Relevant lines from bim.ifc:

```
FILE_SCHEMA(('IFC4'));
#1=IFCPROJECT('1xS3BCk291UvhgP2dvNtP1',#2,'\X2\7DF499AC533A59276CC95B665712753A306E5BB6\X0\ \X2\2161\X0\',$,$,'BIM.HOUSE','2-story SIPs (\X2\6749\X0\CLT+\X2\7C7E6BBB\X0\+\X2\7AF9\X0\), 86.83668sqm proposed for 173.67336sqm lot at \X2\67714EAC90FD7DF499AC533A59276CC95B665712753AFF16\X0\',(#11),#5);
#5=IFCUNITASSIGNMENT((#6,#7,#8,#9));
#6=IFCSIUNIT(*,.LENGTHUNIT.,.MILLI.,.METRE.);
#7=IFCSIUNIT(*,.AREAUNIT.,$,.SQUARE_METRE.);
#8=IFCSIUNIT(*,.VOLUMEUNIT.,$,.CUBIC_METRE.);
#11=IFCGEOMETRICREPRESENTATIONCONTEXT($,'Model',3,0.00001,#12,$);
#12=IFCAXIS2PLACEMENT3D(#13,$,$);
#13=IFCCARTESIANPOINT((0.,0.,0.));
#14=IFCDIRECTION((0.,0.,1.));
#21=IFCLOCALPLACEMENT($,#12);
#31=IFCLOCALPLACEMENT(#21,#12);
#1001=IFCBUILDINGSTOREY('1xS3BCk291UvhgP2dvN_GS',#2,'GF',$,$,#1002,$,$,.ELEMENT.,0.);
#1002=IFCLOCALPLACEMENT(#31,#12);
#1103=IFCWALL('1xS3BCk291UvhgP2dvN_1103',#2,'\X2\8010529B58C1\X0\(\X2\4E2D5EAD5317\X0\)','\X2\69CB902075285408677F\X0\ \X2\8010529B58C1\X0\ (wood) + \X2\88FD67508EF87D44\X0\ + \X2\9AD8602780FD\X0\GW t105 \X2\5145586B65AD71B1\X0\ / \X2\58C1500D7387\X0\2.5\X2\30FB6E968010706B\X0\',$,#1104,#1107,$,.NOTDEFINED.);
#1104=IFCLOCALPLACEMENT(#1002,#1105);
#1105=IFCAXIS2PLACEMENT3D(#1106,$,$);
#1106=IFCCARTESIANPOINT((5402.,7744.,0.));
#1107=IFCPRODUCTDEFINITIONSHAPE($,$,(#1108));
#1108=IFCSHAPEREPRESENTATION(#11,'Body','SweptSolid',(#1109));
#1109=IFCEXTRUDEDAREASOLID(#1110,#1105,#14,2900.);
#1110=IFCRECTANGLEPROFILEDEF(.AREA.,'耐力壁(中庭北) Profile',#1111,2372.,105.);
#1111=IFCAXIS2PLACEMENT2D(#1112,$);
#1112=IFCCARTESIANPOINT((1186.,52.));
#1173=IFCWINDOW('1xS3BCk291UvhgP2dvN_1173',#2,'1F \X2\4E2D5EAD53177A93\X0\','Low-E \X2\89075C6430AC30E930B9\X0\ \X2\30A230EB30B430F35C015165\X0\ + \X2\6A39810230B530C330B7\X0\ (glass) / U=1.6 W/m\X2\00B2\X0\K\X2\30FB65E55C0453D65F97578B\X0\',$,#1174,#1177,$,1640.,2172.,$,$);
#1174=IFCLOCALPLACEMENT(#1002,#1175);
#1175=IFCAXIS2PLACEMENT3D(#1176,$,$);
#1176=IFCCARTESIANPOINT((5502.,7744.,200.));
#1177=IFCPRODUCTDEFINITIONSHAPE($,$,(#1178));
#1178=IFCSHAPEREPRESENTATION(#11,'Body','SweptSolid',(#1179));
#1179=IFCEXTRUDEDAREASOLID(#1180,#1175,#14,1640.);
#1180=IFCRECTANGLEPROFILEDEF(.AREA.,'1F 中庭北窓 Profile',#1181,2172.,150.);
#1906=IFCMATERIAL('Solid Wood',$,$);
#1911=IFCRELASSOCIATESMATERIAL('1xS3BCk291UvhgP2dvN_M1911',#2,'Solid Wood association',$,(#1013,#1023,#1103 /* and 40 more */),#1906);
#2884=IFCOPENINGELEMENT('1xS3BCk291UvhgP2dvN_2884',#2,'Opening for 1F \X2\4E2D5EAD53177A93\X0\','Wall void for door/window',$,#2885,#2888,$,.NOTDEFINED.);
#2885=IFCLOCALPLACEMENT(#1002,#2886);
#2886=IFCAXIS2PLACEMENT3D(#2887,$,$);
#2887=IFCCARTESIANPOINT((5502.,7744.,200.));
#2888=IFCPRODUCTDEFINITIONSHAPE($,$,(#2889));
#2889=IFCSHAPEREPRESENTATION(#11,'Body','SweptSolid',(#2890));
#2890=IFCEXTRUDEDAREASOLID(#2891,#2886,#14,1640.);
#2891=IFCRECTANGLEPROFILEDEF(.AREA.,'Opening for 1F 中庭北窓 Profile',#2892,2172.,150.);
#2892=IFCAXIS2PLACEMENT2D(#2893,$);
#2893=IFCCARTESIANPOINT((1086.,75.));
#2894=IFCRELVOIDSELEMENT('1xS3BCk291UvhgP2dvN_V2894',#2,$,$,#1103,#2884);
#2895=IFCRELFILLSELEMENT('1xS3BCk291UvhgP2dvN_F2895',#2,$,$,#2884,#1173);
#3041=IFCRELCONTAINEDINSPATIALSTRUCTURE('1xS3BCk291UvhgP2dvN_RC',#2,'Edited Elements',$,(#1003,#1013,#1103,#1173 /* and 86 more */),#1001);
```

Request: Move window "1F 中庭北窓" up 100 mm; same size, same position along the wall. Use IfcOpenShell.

```python
import numpy as np
import ifcopenshell
import ifcopenshell.api.geometry
import ifcopenshell.util.placement
import ifcopenshell.util.unit

model = ifcopenshell.open("bim.ifc")
unit_scale = ifcopenshell.util.unit.calculate_unit_scale(model)

window = model.by_id(1173)
opening = window.FillsVoids[0].RelatingOpeningElement
dz = 0.1 / unit_scale

shift = np.array([0.0, 0.0, dz])
# The window is not placed relative to its opening, so move both.
for product in (opening, window):
    matrix = ifcopenshell.util.placement.get_local_placement(product.ObjectPlacement)
    matrix[:3, 3] += shift
    ifcopenshell.api.geometry.edit_object_placement(model, product=product, matrix=matrix, is_si=False)

print(f"moved by {dz * unit_scale:+.3f} m")

model.write("bim_updated.ifc")
```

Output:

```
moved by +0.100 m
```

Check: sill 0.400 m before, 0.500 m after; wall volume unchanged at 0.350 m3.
